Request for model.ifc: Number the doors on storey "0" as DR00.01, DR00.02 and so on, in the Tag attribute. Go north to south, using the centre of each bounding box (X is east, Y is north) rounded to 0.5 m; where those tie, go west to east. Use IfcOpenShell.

First a look at what the model holds.

```python
import ifcopenshell
import ifcopenshell.util.element
import ifcopenshell.util.placement

model = ifcopenshell.open("model.ifc")
print(model.schema)
storey = next(s for s in model.by_type("IfcBuildingStorey") if s.Name == "0")
doors = [e for e in ifcopenshell.util.element.get_decomposition(storey) if e.is_a("IfcDoor")]
for e in sorted(doors, key=lambda e: e.id()):
    origin = ifcopenshell.util.placement.get_local_placement(e.ObjectPlacement)[:3, 3]
    print(e.id(), e.Tag, e.Name, origin.round(2) + 0.0, sep=" | ")
```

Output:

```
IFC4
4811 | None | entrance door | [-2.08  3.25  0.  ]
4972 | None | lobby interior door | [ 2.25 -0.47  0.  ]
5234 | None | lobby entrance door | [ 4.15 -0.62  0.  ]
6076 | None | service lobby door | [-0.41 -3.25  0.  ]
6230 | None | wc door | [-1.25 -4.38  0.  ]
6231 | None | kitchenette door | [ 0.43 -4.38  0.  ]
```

```python
import ifcopenshell
import ifcopenshell.geom
import ifcopenshell.util.element
import ifcopenshell.util.shape

model = ifcopenshell.open("model.ifc")
settings = ifcopenshell.geom.settings()
settings.set("use-world-coords", True)


def centre(element):
    shape = ifcopenshell.geom.create_shape(settings, element)
    return ifcopenshell.util.shape.get_bbox_centroid(shape.geometry)


storey = next(s for s in model.by_type("IfcBuildingStorey") if s.Name == "0")
doors = [e for e in ifcopenshell.util.element.get_decomposition(storey) if e.is_a("IfcDoor")]

# Insertion points can sit at a corner or the storey origin, so sort by the geometry (in metres).
centres = {e: centre(e) for e in doors}
doors.sort(key=lambda e: (-round(centres[e][1] / 0.5), centres[e][0]))

for i, e in enumerate(doors, start=1):
    number = f"DR00.{i:02d}"
    e.Tag = number
    print(e.id(), number)

model.write("model_edited.ifc")
```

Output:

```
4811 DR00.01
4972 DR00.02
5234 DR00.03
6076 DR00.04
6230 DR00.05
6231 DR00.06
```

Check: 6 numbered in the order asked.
